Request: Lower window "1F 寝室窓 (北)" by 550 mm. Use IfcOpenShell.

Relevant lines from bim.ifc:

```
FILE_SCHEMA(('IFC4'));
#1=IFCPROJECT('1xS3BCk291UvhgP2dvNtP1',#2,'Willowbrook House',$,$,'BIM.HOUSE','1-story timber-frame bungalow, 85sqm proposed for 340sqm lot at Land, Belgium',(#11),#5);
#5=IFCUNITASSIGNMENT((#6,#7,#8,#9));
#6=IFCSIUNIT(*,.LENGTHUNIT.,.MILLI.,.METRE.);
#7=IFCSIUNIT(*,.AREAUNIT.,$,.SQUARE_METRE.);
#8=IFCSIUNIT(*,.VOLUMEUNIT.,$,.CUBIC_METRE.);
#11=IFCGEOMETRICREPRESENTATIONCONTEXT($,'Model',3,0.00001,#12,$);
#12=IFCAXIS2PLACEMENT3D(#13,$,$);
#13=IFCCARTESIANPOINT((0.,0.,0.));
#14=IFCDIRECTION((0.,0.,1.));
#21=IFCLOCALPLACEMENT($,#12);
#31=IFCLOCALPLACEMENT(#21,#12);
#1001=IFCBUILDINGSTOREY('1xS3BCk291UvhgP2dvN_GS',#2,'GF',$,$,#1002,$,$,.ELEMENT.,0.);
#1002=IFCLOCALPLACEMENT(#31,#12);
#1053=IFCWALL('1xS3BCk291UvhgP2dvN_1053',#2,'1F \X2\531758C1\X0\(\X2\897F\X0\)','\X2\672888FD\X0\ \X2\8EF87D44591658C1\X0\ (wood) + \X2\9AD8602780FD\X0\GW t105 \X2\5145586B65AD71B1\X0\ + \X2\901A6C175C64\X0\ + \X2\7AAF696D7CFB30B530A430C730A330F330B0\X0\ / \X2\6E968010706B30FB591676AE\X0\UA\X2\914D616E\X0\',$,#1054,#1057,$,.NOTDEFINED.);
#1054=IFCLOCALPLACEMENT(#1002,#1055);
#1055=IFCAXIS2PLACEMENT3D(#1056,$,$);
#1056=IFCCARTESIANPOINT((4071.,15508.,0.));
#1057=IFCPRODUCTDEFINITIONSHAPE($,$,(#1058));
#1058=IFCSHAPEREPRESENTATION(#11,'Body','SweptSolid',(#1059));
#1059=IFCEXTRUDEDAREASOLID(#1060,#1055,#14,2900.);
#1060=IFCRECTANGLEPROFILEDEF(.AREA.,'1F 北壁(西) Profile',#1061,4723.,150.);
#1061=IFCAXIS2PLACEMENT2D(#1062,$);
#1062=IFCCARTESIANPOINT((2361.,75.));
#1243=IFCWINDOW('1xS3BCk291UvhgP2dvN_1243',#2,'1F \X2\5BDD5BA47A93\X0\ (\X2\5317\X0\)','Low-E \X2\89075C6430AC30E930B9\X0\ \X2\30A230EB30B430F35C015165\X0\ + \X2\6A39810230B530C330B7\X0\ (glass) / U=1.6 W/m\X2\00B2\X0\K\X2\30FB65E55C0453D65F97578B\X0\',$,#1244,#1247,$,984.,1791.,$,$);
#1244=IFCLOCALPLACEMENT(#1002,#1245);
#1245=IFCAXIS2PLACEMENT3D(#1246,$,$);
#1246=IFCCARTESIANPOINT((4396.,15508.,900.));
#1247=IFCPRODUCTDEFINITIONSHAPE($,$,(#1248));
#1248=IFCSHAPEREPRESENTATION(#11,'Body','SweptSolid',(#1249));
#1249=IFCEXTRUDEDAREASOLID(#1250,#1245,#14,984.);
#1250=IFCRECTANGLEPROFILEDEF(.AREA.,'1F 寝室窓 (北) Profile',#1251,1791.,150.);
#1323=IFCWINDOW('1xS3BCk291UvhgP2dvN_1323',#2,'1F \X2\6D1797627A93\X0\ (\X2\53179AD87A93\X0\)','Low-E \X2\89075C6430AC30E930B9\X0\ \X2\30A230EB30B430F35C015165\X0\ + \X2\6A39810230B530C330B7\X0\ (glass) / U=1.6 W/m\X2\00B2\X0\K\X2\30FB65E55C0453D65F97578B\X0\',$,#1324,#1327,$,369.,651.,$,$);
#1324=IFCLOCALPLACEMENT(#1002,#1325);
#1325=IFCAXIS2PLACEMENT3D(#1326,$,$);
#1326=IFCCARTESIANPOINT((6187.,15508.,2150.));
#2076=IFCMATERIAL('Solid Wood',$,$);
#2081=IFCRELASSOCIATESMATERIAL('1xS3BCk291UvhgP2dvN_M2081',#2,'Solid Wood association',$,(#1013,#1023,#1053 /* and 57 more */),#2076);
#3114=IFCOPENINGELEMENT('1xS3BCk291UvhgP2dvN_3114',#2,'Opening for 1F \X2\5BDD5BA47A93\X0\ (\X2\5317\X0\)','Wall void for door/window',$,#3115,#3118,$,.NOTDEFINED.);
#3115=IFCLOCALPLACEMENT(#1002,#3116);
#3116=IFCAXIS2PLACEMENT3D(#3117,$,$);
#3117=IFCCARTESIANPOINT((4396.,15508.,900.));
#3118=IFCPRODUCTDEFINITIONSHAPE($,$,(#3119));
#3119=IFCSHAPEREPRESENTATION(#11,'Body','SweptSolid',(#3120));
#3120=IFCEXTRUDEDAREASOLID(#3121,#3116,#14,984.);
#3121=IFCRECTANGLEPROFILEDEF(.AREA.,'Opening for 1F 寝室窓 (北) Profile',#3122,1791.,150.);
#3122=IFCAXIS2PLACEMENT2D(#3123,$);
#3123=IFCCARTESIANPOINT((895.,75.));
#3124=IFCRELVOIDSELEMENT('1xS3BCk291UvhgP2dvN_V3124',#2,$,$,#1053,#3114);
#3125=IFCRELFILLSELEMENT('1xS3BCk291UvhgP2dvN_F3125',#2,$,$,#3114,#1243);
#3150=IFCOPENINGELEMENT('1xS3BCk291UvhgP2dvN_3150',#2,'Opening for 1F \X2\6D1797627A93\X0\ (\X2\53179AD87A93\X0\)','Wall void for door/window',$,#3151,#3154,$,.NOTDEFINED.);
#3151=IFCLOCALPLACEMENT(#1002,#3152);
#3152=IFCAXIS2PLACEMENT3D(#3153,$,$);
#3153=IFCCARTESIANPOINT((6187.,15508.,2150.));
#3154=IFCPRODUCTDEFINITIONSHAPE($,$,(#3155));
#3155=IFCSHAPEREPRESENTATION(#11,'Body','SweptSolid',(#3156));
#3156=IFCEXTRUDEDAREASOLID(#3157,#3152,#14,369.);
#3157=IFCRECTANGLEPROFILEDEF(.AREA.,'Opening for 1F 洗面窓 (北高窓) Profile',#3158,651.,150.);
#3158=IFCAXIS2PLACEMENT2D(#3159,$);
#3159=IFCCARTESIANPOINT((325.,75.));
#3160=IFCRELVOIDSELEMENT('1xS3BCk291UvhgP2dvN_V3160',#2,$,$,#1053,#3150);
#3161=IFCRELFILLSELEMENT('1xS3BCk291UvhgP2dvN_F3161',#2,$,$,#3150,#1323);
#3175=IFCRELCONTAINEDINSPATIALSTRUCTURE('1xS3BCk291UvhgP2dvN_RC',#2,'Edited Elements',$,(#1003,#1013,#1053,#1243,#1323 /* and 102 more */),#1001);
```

```python
import numpy as np
import ifcopenshell
import ifcopenshell.api.geometry
import ifcopenshell.util.placement
import ifcopenshell.util.unit

model = ifcopenshell.open("bim.ifc")
unit_scale = ifcopenshell.util.unit.calculate_unit_scale(model)

window = model.by_id(1243)
opening = window.FillsVoids[0].RelatingOpeningElement
dz = -550.0

shift = np.array([0.0, 0.0, dz])
# The window is not placed relative to its opening, so move both.
for product in (opening, window):
    matrix = ifcopenshell.util.placement.get_local_placement(product.ObjectPlacement)
    matrix[:3, 3] += shift
    ifcopenshell.api.geometry.edit_object_placement(model, product=product, matrix=matrix, is_si=False)

print(f"moved by {dz * unit_scale:+.3f} m")

model.write("bim_updated.ifc")
```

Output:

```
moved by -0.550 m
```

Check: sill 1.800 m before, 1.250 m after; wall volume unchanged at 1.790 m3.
